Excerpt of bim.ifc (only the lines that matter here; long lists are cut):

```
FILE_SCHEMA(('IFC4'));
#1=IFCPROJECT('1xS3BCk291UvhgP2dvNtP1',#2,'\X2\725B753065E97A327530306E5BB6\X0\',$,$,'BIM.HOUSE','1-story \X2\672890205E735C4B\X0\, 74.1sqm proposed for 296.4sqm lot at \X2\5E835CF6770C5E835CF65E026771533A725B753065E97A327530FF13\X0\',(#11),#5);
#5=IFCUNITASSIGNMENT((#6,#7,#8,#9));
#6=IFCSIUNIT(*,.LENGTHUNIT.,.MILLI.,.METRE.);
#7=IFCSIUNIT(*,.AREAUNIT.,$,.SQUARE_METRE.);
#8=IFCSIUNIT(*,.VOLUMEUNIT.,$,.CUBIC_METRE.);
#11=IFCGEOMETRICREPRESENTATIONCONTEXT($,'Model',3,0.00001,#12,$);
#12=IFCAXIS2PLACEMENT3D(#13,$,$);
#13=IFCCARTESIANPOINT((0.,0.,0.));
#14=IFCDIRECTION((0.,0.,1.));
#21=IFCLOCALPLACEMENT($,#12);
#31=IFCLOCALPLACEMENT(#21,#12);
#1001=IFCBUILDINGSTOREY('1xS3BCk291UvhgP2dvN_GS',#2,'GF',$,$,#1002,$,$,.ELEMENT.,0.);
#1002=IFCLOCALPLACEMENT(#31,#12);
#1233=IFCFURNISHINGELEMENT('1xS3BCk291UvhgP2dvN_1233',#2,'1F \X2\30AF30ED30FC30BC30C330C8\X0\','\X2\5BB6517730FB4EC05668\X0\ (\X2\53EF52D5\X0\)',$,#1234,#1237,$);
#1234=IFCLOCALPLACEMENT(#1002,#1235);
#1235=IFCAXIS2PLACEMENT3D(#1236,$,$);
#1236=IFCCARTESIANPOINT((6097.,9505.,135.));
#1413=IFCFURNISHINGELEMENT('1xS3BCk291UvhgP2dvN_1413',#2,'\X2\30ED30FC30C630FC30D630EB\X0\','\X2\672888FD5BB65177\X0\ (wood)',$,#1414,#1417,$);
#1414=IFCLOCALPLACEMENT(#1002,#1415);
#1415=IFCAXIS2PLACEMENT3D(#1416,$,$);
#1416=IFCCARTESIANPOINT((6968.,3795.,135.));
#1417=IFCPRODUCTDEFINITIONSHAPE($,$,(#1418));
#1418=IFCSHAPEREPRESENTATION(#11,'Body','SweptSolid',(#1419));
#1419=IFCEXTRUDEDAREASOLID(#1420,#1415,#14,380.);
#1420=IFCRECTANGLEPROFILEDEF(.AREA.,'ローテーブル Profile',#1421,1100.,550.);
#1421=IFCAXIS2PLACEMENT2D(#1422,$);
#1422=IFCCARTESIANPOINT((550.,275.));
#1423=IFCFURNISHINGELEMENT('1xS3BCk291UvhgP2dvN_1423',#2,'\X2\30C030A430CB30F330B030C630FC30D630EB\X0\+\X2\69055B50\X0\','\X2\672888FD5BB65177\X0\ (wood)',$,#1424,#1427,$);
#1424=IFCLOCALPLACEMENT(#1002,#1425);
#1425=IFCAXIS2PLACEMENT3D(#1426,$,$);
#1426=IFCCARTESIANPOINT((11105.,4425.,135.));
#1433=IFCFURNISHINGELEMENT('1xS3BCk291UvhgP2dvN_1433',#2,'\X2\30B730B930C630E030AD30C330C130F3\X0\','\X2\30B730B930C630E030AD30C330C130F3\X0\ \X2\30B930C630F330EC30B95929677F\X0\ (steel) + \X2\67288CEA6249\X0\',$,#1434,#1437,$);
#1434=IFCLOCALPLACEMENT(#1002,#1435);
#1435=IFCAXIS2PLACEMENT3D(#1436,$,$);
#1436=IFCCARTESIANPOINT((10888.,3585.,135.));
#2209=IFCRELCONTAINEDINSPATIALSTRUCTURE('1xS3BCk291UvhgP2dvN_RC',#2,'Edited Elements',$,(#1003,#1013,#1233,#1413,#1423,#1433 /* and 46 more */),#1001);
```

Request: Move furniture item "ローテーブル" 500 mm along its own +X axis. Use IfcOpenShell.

```python
import ifcopenshell
import ifcopenshell.api.geometry
import ifcopenshell.util.placement
import ifcopenshell.util.unit

model = ifcopenshell.open("bim.ifc")
unit_scale = ifcopenshell.util.unit.calculate_unit_scale(model)

item = model.by_id(1413)
matrix = ifcopenshell.util.placement.get_local_placement(item.ObjectPlacement)
matrix[:3, 3] += matrix[:3, 0] * 0.5 / unit_scale
ifcopenshell.api.geometry.edit_object_placement(model, product=item, matrix=matrix, is_si=False)

print(ifcopenshell.util.placement.get_local_placement(item.ObjectPlacement).round(3) + 0.0)

model.write("bim_updated.ifc")
```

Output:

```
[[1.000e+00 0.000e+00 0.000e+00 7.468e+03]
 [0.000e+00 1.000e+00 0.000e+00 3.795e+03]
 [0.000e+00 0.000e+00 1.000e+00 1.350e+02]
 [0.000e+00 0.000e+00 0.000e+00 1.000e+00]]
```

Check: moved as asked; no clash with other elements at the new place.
